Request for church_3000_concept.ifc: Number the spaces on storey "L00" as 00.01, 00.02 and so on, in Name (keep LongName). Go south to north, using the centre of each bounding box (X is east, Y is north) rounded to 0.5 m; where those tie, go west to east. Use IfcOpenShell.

First a look at what the model holds.

```python
import ifcopenshell
import ifcopenshell.util.element
import ifcopenshell.util.placement

model = ifcopenshell.open("church_3000_concept.ifc")
print(model.schema)
storey = next(s for s in model.by_type("IfcBuildingStorey") if s.Name == "L00")
spaces = [e for e in ifcopenshell.util.element.get_decomposition(storey) if e.is_a("IfcSpace")]
for e in sorted(spaces, key=lambda e: e.id()):
    origin = ifcopenshell.util.placement.get_local_placement(e.ObjectPlacement)[:3, 3]
    print(e.id(), e.Name, e.LongName, origin.round(2) + 0.0, sep=" | ")
```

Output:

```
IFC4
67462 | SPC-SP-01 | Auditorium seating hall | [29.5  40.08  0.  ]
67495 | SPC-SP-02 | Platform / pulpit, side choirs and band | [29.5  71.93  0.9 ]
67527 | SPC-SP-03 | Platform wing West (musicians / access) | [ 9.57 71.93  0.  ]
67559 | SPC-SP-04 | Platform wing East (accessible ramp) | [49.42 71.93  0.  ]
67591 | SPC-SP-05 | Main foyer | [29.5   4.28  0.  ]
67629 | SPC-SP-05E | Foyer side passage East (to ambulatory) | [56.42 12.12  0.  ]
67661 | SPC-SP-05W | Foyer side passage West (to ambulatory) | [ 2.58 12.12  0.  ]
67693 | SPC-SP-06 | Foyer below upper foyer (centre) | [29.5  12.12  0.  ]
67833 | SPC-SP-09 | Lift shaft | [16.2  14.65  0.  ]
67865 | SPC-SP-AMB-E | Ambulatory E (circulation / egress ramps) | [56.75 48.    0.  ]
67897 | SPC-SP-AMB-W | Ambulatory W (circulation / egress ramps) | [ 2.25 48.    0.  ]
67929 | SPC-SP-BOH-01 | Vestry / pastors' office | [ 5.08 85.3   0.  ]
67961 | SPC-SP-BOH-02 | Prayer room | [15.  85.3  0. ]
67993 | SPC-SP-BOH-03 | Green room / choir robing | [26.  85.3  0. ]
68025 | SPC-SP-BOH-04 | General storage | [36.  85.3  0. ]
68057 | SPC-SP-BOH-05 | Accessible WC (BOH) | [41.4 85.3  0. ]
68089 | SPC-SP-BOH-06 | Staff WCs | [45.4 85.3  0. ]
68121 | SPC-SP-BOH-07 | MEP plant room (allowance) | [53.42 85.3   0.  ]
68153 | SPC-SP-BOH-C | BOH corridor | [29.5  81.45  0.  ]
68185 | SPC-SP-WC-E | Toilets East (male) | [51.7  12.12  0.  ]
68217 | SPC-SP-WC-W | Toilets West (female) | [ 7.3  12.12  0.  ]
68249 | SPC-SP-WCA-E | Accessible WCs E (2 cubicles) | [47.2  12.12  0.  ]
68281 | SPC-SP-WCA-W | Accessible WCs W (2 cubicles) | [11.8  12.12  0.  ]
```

```python
import ifcopenshell
import ifcopenshell.geom
import ifcopenshell.util.element
import ifcopenshell.util.shape

model = ifcopenshell.open("church_3000_concept.ifc")
settings = ifcopenshell.geom.settings()
settings.set("use-world-coords", True)


def centre(element):
    shape = ifcopenshell.geom.create_shape(settings, element)
    return ifcopenshell.util.shape.get_bbox_centroid(shape.geometry)


storey = next(s for s in model.by_type("IfcBuildingStorey") if s.Name == "L00")
spaces = [e for e in ifcopenshell.util.element.get_decomposition(storey) if e.is_a("IfcSpace")]

# Insertion points can sit at a corner or the storey origin, so sort by the geometry (in metres).
centres = {e: centre(e) for e in spaces}
spaces.sort(key=lambda e: (round(centres[e][1] / 0.5), centres[e][0]))

for i, e in enumerate(spaces, start=1):
    number = f"00.{i:02d}"
    e.Name = number
    print(e.id(), number)

model.write("church_3000_concept_edited.ifc")
```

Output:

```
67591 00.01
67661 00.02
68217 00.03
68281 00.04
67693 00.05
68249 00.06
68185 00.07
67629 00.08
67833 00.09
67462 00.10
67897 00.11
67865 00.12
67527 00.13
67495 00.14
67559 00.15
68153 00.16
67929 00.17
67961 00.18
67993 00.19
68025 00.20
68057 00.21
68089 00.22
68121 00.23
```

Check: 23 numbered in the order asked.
